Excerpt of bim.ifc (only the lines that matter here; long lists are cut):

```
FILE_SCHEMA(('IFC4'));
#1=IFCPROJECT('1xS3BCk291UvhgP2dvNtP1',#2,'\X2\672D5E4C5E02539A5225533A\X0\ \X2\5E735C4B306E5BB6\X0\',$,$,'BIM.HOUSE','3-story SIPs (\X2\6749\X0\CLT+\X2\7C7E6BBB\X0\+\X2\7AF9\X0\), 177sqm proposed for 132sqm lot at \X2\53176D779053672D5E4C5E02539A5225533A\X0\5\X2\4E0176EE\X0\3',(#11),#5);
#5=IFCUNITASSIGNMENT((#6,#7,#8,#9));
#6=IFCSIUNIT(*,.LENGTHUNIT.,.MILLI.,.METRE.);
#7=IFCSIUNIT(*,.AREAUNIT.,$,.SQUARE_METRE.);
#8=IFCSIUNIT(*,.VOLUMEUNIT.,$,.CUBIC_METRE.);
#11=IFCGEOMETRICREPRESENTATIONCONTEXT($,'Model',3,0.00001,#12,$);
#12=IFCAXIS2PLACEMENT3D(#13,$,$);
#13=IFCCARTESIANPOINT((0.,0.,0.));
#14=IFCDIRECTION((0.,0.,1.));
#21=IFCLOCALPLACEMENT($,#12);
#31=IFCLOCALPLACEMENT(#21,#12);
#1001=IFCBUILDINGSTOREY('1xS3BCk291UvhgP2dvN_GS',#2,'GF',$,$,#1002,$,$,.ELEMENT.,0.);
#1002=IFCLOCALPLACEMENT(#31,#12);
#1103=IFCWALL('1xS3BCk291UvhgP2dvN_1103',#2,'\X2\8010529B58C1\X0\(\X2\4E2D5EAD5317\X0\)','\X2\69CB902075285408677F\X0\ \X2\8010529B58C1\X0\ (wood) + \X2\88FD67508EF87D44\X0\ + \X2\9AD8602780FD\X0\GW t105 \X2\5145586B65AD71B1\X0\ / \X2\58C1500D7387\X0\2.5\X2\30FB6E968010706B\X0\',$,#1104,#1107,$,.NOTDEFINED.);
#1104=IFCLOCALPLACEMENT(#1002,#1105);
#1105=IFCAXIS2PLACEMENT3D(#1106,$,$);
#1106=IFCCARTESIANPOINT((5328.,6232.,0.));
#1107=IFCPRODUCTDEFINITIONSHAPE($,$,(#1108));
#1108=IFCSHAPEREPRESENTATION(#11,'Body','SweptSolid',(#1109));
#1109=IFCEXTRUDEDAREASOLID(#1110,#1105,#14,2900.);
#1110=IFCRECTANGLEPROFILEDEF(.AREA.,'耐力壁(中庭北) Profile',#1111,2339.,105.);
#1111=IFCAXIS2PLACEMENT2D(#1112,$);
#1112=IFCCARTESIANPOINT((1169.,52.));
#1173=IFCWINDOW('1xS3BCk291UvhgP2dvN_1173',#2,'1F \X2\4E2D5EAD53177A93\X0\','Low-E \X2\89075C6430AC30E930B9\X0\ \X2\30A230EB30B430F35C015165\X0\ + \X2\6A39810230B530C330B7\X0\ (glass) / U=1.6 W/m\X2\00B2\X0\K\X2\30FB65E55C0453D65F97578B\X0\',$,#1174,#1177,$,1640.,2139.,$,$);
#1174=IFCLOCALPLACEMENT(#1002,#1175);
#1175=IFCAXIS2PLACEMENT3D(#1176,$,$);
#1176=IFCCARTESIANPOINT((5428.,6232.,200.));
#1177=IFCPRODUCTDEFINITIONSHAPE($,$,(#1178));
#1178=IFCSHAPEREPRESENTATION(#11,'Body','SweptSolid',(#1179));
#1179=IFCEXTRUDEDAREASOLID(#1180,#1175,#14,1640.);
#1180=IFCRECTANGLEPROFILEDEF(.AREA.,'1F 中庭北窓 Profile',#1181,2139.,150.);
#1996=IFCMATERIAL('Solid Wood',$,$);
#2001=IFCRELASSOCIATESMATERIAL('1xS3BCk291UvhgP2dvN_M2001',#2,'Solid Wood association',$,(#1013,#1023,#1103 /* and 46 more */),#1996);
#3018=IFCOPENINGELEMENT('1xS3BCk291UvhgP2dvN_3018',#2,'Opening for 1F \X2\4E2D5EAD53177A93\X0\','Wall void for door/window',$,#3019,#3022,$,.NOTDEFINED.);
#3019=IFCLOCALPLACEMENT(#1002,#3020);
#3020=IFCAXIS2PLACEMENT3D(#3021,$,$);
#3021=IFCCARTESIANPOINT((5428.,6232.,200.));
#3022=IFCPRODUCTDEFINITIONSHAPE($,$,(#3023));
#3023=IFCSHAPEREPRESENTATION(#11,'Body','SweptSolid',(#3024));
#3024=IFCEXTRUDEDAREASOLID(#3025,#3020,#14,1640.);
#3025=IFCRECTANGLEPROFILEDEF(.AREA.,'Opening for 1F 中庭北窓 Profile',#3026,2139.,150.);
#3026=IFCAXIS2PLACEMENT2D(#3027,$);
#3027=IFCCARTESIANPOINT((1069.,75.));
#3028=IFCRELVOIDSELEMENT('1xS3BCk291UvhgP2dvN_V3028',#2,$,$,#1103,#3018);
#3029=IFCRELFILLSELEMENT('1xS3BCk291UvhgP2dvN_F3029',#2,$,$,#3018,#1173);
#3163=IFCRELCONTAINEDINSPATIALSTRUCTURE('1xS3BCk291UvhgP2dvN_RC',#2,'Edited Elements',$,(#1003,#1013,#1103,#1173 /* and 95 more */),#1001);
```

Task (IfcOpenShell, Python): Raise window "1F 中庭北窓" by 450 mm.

```python
import numpy as np
import ifcopenshell
import ifcopenshell.api.geometry
import ifcopenshell.util.placement
import ifcopenshell.util.unit

model = ifcopenshell.open("bim.ifc")
unit_scale = ifcopenshell.util.unit.calculate_unit_scale(model)

window = model.by_guid("1xS3BCk291UvhgP2dvN_1173")
opening = window.FillsVoids[0].RelatingOpeningElement
dz = 0.45 / unit_scale

shift = np.array([0.0, 0.0, dz])
# The window is not placed relative to its opening, so move both.
for product in (opening, window):
    matrix = ifcopenshell.util.placement.get_local_placement(product.ObjectPlacement)
    matrix[:3, 3] += shift
    ifcopenshell.api.geometry.edit_object_placement(model, product=product, matrix=matrix, is_si=False)

print(f"moved by {dz * unit_scale:+.3f} m")

model.write("bim_v2.ifc")
```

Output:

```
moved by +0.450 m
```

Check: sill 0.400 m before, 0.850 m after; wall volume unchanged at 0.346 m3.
